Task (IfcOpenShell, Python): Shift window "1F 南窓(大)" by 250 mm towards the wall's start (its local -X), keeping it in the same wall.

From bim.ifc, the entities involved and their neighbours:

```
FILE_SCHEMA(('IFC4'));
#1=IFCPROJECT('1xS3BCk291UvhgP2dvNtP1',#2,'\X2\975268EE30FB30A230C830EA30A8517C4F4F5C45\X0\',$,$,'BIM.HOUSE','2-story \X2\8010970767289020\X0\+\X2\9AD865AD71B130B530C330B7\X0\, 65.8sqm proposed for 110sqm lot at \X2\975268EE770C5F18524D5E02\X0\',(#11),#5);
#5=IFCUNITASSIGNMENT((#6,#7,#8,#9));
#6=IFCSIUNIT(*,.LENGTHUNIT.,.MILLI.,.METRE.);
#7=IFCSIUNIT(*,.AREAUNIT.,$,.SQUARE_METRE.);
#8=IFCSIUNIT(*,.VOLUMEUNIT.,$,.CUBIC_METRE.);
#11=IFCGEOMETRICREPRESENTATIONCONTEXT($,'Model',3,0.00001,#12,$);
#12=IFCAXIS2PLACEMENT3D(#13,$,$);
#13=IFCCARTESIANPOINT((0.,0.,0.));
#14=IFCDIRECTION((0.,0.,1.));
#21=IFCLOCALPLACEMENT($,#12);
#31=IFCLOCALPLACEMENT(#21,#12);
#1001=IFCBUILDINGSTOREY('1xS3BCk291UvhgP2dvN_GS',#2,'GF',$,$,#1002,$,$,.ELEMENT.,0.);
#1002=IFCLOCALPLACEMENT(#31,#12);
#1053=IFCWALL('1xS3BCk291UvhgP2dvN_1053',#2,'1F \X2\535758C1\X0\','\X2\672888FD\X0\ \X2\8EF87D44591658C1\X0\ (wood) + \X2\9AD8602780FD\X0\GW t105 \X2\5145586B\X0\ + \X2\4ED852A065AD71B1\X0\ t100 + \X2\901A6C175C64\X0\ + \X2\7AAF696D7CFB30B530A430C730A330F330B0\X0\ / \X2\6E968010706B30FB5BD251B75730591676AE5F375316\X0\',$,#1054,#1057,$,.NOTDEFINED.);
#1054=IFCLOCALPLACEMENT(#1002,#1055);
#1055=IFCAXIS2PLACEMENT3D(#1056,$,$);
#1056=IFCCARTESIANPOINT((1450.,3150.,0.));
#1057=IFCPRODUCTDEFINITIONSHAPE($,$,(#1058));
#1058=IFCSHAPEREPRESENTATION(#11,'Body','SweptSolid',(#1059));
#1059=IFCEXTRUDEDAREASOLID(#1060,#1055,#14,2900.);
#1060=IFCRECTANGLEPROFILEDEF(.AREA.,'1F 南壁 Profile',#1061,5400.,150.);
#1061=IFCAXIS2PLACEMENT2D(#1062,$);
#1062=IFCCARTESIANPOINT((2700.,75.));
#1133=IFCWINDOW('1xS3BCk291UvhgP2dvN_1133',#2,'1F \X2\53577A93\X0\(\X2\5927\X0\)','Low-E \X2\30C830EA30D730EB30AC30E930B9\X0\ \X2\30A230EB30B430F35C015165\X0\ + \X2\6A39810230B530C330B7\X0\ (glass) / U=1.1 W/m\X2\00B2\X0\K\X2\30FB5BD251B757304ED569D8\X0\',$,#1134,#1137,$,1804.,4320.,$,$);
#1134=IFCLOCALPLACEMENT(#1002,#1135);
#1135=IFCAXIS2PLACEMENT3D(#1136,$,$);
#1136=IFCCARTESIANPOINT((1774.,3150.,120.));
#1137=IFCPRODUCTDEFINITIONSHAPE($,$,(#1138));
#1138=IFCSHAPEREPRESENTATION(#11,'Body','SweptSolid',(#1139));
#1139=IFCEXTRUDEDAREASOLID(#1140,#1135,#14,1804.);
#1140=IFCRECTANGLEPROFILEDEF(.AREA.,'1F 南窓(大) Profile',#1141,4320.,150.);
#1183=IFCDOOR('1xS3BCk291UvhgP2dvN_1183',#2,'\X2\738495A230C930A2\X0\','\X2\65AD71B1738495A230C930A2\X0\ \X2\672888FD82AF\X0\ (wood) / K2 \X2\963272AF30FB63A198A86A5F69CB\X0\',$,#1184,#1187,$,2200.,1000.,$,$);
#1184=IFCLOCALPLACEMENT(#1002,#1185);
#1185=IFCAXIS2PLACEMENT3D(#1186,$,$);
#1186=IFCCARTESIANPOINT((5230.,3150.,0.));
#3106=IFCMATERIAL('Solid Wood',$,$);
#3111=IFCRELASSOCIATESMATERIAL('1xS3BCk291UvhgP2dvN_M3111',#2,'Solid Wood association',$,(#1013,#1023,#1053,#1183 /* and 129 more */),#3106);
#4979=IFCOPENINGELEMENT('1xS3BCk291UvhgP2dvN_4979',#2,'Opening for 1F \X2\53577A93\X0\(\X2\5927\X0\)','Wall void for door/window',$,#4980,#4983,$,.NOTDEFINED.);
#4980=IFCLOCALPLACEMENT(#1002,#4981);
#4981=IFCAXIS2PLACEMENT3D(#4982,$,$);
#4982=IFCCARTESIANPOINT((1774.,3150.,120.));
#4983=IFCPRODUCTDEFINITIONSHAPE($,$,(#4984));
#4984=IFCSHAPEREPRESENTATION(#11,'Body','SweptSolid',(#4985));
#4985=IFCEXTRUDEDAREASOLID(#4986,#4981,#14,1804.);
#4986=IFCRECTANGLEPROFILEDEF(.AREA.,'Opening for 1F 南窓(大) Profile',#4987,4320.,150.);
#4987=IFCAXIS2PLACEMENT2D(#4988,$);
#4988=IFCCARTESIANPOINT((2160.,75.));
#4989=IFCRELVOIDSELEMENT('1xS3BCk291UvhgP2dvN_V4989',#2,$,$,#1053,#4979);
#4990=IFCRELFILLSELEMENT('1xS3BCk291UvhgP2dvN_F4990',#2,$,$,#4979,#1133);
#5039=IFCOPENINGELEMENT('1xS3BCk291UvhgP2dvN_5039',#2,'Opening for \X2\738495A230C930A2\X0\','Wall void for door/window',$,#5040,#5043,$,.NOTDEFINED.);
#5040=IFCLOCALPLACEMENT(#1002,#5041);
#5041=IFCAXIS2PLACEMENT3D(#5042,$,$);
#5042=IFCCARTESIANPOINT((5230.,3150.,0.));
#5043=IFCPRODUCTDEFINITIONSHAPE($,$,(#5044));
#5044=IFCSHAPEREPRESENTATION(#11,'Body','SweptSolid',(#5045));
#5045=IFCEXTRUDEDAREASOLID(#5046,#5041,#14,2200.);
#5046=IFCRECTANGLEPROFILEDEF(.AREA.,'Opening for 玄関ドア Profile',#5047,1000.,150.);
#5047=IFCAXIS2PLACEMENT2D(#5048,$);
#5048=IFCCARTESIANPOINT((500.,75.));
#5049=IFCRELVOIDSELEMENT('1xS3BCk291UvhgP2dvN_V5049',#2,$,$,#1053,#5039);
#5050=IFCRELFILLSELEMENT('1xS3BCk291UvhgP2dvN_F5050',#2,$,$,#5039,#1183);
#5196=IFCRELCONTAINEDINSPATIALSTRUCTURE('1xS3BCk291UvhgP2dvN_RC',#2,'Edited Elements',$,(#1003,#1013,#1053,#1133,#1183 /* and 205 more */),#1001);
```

```python
import ifcopenshell
import ifcopenshell.api.geometry
import ifcopenshell.util.placement
import ifcopenshell.util.unit

model = ifcopenshell.open("bim.ifc")
unit_scale = ifcopenshell.util.unit.calculate_unit_scale(model)

window = model.by_guid("1xS3BCk291UvhgP2dvN_1133")
opening = window.FillsVoids[0].RelatingOpeningElement
wall = opening.VoidsElements[0].RelatingBuildingElement

wall_matrix = ifcopenshell.util.placement.get_local_placement(wall.ObjectPlacement)
shift = wall_matrix[:3, 0] * -0.25 / unit_scale
before = ifcopenshell.util.placement.get_local_placement(window.ObjectPlacement)[:3, 3].copy()

# The window is not placed relative to its opening, so move both.
for product in (opening, window):
    matrix = ifcopenshell.util.placement.get_local_placement(product.ObjectPlacement)
    matrix[:3, 3] += shift
    ifcopenshell.api.geometry.edit_object_placement(model, product=product, matrix=matrix, is_si=False)

after = ifcopenshell.util.placement.get_local_placement(window.ObjectPlacement)[:3, 3]
print("window moved by", (after - before).round(3) + 0.0)

model.write("bim_edited.ifc")
```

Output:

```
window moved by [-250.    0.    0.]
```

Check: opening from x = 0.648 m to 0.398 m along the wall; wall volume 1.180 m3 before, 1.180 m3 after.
